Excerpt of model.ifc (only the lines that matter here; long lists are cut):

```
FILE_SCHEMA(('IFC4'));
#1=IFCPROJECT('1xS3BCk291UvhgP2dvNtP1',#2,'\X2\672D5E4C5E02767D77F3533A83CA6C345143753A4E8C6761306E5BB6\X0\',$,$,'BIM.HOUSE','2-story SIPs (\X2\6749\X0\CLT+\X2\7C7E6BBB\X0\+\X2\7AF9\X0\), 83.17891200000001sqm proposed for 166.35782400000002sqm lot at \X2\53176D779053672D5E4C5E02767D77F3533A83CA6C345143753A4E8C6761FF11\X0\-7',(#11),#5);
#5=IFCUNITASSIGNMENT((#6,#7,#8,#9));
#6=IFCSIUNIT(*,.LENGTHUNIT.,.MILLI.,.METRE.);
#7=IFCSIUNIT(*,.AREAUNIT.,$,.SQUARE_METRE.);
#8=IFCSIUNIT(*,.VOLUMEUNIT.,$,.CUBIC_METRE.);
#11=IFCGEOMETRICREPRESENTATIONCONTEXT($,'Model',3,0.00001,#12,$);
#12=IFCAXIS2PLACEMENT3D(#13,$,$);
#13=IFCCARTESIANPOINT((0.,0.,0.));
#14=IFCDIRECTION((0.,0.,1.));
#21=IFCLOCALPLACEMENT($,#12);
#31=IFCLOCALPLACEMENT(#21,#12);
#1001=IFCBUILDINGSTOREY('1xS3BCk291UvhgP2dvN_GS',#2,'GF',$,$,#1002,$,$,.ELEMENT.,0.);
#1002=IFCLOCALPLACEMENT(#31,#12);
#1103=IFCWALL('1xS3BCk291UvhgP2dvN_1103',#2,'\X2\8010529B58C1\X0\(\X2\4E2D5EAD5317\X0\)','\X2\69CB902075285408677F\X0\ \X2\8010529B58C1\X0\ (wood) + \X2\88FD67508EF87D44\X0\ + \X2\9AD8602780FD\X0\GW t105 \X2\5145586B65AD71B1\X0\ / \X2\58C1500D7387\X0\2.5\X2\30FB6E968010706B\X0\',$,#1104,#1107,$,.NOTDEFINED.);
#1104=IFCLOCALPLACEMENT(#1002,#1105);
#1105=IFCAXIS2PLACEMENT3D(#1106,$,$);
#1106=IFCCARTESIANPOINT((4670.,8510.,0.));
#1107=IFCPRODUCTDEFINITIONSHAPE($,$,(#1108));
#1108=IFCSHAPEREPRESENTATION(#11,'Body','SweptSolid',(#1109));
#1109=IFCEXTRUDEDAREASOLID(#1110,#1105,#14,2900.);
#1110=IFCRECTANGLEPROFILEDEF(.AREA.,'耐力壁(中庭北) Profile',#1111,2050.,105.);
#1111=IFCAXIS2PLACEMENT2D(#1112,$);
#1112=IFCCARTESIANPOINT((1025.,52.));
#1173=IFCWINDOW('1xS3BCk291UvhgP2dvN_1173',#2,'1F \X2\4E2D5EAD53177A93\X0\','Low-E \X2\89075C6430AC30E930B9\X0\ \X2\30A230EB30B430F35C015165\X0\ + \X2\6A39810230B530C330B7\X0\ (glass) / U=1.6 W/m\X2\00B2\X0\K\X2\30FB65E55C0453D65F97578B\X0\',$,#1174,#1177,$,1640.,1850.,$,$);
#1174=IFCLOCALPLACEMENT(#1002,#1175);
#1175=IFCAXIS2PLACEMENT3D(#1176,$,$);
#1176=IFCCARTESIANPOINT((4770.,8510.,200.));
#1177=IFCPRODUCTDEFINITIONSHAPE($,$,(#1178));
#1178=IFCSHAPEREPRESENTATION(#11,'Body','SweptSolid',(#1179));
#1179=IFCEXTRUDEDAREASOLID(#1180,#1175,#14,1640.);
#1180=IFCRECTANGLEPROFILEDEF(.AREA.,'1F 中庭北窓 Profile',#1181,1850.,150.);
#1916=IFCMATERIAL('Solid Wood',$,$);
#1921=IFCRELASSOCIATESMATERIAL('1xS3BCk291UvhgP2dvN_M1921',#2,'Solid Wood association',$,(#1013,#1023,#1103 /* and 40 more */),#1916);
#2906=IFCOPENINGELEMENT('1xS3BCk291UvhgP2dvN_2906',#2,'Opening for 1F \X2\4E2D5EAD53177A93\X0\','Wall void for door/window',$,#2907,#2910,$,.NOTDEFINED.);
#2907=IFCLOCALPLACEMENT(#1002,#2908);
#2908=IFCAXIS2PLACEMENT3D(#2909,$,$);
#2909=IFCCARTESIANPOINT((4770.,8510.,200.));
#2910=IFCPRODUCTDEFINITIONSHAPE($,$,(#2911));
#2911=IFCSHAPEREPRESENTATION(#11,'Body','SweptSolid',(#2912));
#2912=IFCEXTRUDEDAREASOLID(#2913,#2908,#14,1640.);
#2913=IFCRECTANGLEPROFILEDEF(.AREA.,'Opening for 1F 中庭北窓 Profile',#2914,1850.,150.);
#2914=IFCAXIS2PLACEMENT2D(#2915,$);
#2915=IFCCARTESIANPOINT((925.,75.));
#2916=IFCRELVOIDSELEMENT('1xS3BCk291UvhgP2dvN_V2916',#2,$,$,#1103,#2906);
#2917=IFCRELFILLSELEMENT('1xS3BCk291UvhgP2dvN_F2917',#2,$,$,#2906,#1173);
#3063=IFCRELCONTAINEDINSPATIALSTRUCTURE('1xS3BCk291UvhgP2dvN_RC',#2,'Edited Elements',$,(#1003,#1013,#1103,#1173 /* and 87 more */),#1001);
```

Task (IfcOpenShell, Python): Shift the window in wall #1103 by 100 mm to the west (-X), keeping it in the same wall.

```python
import ifcopenshell
import ifcopenshell.api.geometry
import ifcopenshell.util.placement

model = ifcopenshell.open("model.ifc")

window = model.by_id(1173)
opening = window.FillsVoids[0].RelatingOpeningElement
wall = opening.VoidsElements[0].RelatingBuildingElement

wall_matrix = ifcopenshell.util.placement.get_local_placement(wall.ObjectPlacement)
shift = wall_matrix[:3, 0] * -100.0
before = ifcopenshell.util.placement.get_local_placement(window.ObjectPlacement)[:3, 3].copy()

# The window is not placed relative to its opening, so move both.
for product in (opening, window):
    matrix = ifcopenshell.util.placement.get_local_placement(product.ObjectPlacement)
    matrix[:3, 3] += shift
    ifcopenshell.api.geometry.edit_object_placement(model, product=product, matrix=matrix, is_si=False)

after = ifcopenshell.util.placement.get_local_placement(window.ObjectPlacement)[:3, 3]
print("window moved by", (after - before).round(3) + 0.0)

model.write("model_rev.ifc")
```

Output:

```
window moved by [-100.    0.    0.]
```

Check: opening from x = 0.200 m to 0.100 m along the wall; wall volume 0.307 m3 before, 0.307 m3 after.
